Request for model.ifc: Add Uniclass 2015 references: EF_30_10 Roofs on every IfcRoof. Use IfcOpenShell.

First a look at what the model holds.

```python
import ifcopenshell

model = ifcopenshell.open("model.ifc")
print(model.schema)
print("classifications:", [c.Name for c in model.by_type("IfcClassification")])
for ifc_class in ("IfcDoor", "IfcRoof", "IfcStair", "IfcWall", "IfcWindow"):
    print(ifc_class, len(model.by_type(ifc_class)))
```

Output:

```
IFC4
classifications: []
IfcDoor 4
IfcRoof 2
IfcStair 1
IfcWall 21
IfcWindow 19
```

```python
import ifcopenshell
import ifcopenshell.api.classification

model = ifcopenshell.open("model.ifc")

system = ifcopenshell.api.classification.add_classification(model, classification="Uniclass 2015")

codes = {
    "IfcRoof": ("EF_30_10", "Roofs"),
}
for ifc_class, (code, name) in codes.items():
    products = model.by_type(ifc_class)
    ifcopenshell.api.classification.add_reference(
        model, products=products, classification=system, identification=code, name=name
    )
    print(code, len(products))

model.write("model-out.ifc")
```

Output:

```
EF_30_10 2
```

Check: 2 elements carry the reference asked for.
